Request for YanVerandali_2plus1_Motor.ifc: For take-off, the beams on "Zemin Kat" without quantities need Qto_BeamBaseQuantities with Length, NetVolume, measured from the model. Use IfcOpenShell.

First a look at what the model holds.

```python
import ifcopenshell
import ifcopenshell.util.element
import ifcopenshell.util.unit

model = ifcopenshell.open("YanVerandali_2plus1_Motor.ifc")
print(model.schema)
for unit_type in ("LENGTHUNIT", "AREAUNIT", "VOLUMEUNIT"):
    print(unit_type, ifcopenshell.util.unit.calculate_unit_scale(model, unit_type))
storey = next(s for s in model.by_type("IfcBuildingStorey") if s.Name == "Zemin Kat")
beams = [e for e in ifcopenshell.util.element.get_decomposition(storey) if e.is_a("IfcBeam")]
for e in sorted(beams, key=lambda e: e.id()):
    print(e.id(), e.is_a(), e.Name, list(ifcopenshell.util.element.get_psets(e, qtos_only=True)), sep=" | ")
```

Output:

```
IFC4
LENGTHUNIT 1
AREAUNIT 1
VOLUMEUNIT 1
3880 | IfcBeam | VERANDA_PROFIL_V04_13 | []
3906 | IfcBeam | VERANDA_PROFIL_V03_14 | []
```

```python
import ifcopenshell
import ifcopenshell.api.pset
import ifcopenshell.geom
import ifcopenshell.util.element
import ifcopenshell.util.shape
import ifcopenshell.util.unit

model = ifcopenshell.open("YanVerandali_2plus1_Motor.ifc")
unit_scale = ifcopenshell.util.unit.calculate_unit_scale(model)
volume_scale = ifcopenshell.util.unit.calculate_unit_scale(model, "VOLUMEUNIT")
settings = ifcopenshell.geom.settings()

storey = next(s for s in model.by_type("IfcBuildingStorey") if s.Name == "Zemin Kat")
beams = [e for e in ifcopenshell.util.element.get_decomposition(storey) if e.is_a("IfcBeam")]

for e in sorted(beams, key=lambda e: e.id()):
    if ifcopenshell.util.element.get_psets(e, qtos_only=True, should_inherit=False):
        continue
    # Geometry comes back in metres, in the element's own axes.
    shape = ifcopenshell.geom.create_shape(settings, e)
    values = {
        "Length": ifcopenshell.util.shape.get_max_xyz(shape.geometry) / unit_scale,
        "NetVolume": ifcopenshell.util.shape.get_volume(shape.geometry) / volume_scale,
    }
    qto = ifcopenshell.api.pset.add_qto(model, product=e, name="Qto_BeamBaseQuantities")
    ifcopenshell.api.pset.edit_qto(model, qto=qto, properties=values)
    print(e.id(), {k: round(v, 3) for k, v in values.items()})

model.write("YanVerandali_2plus1_Motor-out.ifc")
```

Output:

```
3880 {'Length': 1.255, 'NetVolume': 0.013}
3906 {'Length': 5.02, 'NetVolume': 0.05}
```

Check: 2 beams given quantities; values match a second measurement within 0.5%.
